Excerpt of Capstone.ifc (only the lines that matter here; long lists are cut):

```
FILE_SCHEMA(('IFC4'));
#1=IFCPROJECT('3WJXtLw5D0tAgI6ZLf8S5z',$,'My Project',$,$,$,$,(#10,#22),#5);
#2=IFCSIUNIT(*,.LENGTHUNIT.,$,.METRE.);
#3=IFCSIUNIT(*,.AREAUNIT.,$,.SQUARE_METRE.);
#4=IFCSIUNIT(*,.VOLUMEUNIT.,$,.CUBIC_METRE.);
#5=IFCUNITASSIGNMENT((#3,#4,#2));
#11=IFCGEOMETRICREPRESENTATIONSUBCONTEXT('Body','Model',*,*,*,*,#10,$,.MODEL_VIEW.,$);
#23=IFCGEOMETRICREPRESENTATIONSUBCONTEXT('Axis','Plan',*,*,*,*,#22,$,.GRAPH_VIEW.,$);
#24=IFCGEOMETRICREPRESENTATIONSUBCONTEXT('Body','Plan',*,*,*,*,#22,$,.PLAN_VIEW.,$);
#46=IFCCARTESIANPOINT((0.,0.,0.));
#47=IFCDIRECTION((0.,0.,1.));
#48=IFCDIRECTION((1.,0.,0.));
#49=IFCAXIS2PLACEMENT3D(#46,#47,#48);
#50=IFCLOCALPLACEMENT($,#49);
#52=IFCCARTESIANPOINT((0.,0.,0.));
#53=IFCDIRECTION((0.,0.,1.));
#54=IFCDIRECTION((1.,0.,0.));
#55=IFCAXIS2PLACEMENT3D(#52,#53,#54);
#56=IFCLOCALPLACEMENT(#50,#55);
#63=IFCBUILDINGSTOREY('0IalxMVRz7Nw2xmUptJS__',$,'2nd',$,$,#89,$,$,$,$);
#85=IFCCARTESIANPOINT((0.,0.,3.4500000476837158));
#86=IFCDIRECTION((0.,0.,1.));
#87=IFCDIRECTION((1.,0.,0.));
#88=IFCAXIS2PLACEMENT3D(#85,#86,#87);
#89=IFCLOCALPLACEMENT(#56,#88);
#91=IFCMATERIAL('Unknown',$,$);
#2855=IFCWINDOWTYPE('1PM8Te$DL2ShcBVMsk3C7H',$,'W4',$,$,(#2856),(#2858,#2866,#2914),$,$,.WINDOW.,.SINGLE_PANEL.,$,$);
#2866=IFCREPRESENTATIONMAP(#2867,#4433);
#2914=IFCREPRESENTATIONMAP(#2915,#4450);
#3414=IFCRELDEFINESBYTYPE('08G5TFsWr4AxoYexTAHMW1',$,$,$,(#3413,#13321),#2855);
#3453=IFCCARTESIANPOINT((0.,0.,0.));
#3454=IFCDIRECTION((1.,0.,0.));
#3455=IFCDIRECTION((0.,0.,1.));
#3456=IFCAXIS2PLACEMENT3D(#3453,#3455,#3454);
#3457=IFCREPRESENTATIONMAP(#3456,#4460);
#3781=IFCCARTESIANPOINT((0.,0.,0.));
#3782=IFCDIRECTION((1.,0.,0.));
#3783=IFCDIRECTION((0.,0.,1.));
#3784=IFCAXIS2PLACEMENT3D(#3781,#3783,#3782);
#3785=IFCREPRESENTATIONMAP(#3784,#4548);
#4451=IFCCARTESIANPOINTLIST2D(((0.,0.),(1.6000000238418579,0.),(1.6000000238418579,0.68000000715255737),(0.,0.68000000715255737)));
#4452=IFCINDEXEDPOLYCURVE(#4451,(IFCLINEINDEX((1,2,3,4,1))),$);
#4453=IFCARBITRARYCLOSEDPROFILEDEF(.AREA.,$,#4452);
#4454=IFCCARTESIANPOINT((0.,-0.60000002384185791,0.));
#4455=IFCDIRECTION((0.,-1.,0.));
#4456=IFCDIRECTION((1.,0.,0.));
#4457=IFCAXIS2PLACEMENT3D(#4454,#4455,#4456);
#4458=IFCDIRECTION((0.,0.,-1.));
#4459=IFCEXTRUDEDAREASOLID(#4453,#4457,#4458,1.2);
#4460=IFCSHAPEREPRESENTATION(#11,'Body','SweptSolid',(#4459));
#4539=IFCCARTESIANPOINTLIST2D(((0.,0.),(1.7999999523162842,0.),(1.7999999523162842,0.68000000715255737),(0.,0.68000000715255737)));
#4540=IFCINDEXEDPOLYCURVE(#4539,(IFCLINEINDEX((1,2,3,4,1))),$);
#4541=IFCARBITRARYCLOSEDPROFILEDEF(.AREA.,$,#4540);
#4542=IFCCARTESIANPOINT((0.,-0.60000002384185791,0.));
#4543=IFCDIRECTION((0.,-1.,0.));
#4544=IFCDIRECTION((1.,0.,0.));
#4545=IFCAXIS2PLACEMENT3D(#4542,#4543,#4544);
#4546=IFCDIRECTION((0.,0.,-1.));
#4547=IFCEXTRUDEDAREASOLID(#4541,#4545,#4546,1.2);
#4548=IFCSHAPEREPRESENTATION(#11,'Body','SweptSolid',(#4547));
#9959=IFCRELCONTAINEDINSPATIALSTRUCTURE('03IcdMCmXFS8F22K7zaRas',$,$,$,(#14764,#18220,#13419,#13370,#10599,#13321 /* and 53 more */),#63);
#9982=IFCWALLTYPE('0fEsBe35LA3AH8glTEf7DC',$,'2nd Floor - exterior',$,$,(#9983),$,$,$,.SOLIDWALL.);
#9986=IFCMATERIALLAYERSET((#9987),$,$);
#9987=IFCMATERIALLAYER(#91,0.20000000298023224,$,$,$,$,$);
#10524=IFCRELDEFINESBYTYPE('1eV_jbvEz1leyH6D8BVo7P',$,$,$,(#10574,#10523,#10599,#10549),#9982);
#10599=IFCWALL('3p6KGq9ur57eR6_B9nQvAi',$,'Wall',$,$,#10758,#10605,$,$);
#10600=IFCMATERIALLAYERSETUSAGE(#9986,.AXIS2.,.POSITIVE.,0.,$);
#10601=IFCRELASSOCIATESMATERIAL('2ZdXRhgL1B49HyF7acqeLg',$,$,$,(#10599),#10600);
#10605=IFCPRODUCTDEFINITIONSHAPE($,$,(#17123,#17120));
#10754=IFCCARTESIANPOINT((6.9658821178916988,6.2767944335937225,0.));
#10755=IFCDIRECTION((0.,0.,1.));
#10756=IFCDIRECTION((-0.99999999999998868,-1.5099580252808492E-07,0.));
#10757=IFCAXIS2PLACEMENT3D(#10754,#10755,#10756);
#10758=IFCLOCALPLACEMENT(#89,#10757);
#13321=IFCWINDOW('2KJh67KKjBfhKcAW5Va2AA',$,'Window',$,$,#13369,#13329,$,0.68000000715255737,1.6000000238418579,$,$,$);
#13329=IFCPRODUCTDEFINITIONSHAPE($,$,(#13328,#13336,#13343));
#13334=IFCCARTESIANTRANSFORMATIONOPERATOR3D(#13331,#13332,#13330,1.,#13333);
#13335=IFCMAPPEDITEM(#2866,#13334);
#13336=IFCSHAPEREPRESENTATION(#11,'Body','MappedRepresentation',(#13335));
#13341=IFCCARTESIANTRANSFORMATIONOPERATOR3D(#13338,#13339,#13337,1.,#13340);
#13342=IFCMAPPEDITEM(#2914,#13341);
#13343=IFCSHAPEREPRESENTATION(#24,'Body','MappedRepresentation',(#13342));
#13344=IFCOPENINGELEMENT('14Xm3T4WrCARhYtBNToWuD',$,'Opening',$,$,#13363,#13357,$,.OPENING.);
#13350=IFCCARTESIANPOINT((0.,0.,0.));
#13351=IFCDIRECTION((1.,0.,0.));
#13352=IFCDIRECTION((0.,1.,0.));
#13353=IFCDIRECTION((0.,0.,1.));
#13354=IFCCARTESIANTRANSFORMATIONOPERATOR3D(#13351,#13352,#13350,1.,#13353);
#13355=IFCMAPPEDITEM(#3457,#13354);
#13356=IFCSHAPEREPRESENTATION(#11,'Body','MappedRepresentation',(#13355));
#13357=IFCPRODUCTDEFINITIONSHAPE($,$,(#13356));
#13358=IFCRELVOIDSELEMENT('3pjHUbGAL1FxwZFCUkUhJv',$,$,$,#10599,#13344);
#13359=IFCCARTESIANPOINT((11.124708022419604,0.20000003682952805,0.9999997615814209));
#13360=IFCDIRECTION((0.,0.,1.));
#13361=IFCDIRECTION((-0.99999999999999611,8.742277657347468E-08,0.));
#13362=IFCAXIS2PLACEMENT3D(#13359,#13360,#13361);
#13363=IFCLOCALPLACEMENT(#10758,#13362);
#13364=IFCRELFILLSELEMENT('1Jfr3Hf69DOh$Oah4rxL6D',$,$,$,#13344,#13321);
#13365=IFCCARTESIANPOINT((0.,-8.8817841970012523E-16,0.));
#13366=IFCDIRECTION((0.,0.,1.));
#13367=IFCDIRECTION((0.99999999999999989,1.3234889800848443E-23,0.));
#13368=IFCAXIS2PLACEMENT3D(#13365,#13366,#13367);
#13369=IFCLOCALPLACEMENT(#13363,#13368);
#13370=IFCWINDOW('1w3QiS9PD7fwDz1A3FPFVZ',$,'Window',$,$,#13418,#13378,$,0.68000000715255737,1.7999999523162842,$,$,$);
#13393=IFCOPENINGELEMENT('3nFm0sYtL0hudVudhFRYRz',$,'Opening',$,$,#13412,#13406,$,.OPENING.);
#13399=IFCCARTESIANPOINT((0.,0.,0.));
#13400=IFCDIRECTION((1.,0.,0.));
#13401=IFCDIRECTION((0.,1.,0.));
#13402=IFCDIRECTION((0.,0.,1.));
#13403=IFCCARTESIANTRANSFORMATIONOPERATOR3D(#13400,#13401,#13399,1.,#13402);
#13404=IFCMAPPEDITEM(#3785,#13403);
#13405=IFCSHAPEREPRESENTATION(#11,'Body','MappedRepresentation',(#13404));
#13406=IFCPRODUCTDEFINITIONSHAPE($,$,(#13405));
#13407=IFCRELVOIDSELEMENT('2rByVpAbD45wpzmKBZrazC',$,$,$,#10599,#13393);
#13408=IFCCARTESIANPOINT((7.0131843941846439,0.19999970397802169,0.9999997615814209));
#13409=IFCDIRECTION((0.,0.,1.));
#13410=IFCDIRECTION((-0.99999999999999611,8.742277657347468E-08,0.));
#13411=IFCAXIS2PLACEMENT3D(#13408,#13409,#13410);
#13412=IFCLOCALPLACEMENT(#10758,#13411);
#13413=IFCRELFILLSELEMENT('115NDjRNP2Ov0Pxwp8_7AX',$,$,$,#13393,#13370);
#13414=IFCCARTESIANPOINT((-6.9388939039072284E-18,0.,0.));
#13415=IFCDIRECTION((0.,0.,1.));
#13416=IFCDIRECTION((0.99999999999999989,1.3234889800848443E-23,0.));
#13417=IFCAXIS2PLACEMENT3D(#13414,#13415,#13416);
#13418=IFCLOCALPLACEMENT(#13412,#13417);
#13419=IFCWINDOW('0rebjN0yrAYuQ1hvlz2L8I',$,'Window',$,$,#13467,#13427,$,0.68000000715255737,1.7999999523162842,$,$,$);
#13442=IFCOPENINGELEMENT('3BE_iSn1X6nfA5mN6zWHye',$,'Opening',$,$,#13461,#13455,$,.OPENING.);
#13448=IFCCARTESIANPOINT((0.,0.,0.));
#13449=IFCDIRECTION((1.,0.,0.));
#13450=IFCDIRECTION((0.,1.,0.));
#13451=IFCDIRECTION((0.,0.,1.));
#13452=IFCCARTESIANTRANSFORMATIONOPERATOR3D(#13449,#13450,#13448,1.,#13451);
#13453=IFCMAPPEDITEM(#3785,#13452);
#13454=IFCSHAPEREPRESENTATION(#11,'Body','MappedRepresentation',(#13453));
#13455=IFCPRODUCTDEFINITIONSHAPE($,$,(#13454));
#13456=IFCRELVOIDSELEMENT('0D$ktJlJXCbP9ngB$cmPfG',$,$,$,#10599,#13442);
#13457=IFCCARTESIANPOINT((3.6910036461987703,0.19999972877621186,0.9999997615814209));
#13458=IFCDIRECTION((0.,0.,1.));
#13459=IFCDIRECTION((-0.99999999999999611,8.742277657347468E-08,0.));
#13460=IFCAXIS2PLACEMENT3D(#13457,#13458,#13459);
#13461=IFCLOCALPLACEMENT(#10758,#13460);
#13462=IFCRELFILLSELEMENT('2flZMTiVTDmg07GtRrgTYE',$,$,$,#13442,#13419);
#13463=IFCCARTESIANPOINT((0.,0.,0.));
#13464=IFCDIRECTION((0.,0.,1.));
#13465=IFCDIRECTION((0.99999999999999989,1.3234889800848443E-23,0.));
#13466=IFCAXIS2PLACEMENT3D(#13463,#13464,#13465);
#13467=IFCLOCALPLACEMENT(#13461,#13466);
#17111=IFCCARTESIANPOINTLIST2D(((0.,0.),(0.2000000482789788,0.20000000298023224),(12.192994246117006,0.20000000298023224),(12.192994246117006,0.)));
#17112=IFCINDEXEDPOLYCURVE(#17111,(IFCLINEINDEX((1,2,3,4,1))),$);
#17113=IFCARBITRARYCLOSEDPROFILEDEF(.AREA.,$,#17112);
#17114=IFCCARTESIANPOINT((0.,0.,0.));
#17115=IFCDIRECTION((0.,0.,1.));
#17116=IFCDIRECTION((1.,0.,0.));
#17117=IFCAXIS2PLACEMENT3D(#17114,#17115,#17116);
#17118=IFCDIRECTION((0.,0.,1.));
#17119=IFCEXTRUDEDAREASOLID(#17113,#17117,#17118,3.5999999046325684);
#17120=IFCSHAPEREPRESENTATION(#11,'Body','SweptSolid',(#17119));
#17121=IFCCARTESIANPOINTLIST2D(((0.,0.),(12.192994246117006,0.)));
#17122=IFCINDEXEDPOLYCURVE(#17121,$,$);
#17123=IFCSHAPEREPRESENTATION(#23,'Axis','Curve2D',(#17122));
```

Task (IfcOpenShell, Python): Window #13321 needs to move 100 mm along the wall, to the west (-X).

```python
import ifcopenshell
import ifcopenshell.api.geometry
import ifcopenshell.util.placement
import ifcopenshell.util.unit

model = ifcopenshell.open("Capstone.ifc")
unit_scale = ifcopenshell.util.unit.calculate_unit_scale(model)

window = model.by_id(13321)
opening = window.FillsVoids[0].RelatingOpeningElement
wall = opening.VoidsElements[0].RelatingBuildingElement

wall_matrix = ifcopenshell.util.placement.get_local_placement(wall.ObjectPlacement)
shift = wall_matrix[:3, 0] * 0.1 / unit_scale
before = ifcopenshell.util.placement.get_local_placement(window.ObjectPlacement)[:3, 3].copy()

# The window is placed relative to its opening, so it follows when the opening moves.
matrix = ifcopenshell.util.placement.get_local_placement(opening.ObjectPlacement)
matrix[:3, 3] += shift
ifcopenshell.api.geometry.edit_object_placement(
    model, product=opening, matrix=matrix, is_si=False, should_transform_children=True
)

after = ifcopenshell.util.placement.get_local_placement(window.ObjectPlacement)[:3, 3]
print("window moved by", (after - before).round(3) + 0.0)

model.write("Capstone_rev.ifc")
```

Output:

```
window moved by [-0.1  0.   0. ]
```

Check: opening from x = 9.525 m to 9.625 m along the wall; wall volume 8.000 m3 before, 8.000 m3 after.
